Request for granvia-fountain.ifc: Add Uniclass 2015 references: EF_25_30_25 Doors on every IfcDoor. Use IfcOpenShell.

First a look at what the model holds.

```python
import ifcopenshell

model = ifcopenshell.open("granvia-fountain.ifc")
print(model.schema)
print("classifications:", [c.Name for c in model.by_type("IfcClassification")])
for ifc_class in ("IfcDoor", "IfcRoof", "IfcStair", "IfcWall", "IfcWindow"):
    print(ifc_class, len(model.by_type(ifc_class)))
```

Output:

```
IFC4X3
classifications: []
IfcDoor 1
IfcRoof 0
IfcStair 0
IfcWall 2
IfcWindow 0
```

```python
import ifcopenshell
import ifcopenshell.api.classification

model = ifcopenshell.open("granvia-fountain.ifc")

system = ifcopenshell.api.classification.add_classification(model, classification="Uniclass 2015")

codes = {
    "IfcDoor": ("EF_25_30_25", "Doors"),
}
for ifc_class, (code, name) in codes.items():
    products = model.by_type(ifc_class)
    ifcopenshell.api.classification.add_reference(
        model, products=products, classification=system, identification=code, name=name
    )
    print(code, len(products))

model.write("granvia-fountain_updated.ifc")
```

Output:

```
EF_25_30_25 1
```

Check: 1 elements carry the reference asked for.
